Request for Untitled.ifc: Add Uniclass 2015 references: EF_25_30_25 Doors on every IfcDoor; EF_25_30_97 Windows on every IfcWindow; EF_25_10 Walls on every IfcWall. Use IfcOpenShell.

First a look at what the model holds.

```python
import ifcopenshell

model = ifcopenshell.open("Untitled.ifc")
print(model.schema)
print("classifications:", [c.Name for c in model.by_type("IfcClassification")])
for ifc_class in ("IfcDoor", "IfcRoof", "IfcStair", "IfcWall", "IfcWindow"):
    print(ifc_class, len(model.by_type(ifc_class)))
```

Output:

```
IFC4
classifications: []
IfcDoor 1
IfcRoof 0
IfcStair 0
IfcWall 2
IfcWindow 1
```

```python
import ifcopenshell
import ifcopenshell.api.classification

model = ifcopenshell.open("Untitled.ifc")

system = ifcopenshell.api.classification.add_classification(model, classification="Uniclass 2015")

codes = {
    "IfcDoor": ("EF_25_30_25", "Doors"),
    "IfcWindow": ("EF_25_30_97", "Windows"),
    "IfcWall": ("EF_25_10", "Walls"),
}
for ifc_class, (code, name) in codes.items():
    products = model.by_type(ifc_class)
    ifcopenshell.api.classification.add_reference(
        model, products=products, classification=system, identification=code, name=name
    )
    print(code, len(products))

model.write("Untitled_v2.ifc")
```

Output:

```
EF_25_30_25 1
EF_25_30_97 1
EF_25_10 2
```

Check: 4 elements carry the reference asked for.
